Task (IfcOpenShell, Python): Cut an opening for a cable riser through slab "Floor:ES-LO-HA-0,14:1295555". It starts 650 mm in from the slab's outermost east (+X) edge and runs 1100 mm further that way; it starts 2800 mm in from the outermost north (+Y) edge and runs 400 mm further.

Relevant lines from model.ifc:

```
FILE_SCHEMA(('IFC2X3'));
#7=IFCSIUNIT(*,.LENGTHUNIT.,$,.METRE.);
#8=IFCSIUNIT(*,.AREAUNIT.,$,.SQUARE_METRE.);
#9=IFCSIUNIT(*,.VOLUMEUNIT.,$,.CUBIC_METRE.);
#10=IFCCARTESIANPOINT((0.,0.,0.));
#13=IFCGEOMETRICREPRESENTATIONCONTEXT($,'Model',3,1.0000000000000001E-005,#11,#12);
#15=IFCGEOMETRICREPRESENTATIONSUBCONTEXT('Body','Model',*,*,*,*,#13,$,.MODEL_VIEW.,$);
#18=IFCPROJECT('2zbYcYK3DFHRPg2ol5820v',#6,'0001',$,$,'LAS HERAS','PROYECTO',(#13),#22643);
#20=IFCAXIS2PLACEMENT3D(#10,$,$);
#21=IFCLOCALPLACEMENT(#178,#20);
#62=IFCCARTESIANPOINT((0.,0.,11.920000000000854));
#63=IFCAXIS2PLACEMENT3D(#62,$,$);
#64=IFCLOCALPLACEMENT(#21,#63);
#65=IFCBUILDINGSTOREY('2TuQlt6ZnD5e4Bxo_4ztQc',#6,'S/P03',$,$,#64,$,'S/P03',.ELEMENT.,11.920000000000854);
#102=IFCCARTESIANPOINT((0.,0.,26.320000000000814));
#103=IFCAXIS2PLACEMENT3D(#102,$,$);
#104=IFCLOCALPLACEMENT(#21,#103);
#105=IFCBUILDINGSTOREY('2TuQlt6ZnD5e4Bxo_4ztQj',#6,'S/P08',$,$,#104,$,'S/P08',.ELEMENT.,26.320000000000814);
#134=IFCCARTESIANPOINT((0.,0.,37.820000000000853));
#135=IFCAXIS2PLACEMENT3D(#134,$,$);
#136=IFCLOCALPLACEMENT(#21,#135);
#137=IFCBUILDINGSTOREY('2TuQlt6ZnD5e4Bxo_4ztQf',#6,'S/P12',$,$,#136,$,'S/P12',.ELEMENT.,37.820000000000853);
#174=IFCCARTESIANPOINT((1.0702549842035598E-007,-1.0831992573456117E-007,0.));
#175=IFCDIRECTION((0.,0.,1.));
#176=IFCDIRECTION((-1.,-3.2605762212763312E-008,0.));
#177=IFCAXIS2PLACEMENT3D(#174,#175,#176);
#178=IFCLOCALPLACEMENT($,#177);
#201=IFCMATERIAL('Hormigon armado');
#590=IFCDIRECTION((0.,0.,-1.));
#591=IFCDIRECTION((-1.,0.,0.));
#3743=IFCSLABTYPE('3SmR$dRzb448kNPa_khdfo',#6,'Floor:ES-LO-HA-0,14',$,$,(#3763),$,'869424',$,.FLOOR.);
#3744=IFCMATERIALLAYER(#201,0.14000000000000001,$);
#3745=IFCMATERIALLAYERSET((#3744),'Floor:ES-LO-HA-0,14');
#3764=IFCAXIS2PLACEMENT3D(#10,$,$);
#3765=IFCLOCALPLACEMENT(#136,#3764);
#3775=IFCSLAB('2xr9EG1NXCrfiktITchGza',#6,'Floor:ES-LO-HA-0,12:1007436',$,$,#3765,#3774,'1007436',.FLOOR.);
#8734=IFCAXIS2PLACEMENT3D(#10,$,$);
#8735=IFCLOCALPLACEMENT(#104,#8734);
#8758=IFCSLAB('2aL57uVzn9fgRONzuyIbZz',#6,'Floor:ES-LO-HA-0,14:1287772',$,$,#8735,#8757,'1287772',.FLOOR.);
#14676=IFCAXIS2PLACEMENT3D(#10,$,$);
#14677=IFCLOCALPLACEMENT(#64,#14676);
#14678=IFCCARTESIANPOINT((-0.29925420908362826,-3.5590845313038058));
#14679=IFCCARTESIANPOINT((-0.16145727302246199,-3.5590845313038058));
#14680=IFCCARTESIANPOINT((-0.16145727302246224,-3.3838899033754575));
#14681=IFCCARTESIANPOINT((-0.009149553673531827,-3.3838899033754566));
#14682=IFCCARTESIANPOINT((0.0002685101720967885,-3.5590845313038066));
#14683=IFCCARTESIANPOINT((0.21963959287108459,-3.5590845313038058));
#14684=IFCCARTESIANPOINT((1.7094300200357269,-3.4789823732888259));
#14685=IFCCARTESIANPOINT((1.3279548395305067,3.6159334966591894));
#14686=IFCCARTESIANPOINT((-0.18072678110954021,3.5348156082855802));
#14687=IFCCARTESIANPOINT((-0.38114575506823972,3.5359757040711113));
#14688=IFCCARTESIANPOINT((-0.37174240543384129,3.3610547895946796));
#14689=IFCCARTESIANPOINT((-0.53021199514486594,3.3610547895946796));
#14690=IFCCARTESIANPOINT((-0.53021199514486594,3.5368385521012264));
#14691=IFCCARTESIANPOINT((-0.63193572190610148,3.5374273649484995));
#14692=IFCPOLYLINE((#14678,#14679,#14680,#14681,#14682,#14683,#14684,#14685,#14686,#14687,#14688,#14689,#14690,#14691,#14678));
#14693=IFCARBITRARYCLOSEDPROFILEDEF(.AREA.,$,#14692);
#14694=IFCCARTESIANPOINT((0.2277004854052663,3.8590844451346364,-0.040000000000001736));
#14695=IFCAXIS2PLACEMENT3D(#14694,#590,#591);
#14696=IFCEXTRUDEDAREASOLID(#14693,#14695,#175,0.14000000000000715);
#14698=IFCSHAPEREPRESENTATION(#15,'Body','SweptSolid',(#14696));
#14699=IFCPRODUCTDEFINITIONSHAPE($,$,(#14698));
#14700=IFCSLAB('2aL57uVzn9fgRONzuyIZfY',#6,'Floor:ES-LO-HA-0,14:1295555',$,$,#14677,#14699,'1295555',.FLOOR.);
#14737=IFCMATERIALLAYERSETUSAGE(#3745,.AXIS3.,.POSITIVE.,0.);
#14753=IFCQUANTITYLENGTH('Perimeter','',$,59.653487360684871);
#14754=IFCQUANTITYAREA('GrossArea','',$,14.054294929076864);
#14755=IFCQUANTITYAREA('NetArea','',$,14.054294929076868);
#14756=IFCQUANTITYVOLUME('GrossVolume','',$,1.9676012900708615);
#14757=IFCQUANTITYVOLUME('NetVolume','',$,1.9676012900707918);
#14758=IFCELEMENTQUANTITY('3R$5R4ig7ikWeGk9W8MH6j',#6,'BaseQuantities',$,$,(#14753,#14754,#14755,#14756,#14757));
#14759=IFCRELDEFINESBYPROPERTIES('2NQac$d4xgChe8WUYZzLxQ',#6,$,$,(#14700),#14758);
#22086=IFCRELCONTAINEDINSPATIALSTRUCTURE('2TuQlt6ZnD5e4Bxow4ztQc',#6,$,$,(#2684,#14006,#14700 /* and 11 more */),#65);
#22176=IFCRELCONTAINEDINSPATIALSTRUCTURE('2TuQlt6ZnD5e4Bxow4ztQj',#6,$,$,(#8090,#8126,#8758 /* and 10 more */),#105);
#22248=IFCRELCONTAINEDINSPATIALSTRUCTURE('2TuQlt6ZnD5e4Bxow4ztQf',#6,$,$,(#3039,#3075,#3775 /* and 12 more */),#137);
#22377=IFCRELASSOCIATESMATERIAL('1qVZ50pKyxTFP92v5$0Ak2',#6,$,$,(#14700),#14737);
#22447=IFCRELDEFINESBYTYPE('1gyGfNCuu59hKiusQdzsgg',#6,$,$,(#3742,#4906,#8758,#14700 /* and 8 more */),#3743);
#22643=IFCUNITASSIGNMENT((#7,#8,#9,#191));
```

```python
import numpy as np
import ifcopenshell
import ifcopenshell.api.feature
import ifcopenshell.api.geometry
import ifcopenshell.api.pset
import ifcopenshell.api.root
import ifcopenshell.geom
import ifcopenshell.util.element
import ifcopenshell.util.placement
import ifcopenshell.util.representation
import ifcopenshell.util.shape
import ifcopenshell.util.unit

model = ifcopenshell.open("model.ifc")
unit_scale = ifcopenshell.util.unit.calculate_unit_scale(model)
area_scale = ifcopenshell.util.unit.calculate_unit_scale(model, "AREAUNIT")
volume_scale = ifcopenshell.util.unit.calculate_unit_scale(model, "VOLUMEUNIT")
settings = ifcopenshell.geom.settings()


def volume(element):
    """Net volume in cubic metres, openings subtracted."""
    shape = ifcopenshell.geom.create_shape(settings, element)
    return ifcopenshell.util.shape.get_volume(shape.geometry)


slab = model.by_id(14700)
before = volume(slab)

# Extent in the slab's own axes, in metres. The edges named are its -X and -Y sides.
slab_shape = ifcopenshell.geom.create_shape(settings, slab)
vertices = ifcopenshell.util.shape.get_vertices(slab_shape.geometry)
x_min, y_min, bottom = vertices.min(axis=0)
top = vertices[:, 2].max()

opening = ifcopenshell.api.root.create_entity(model, ifc_class="IfcOpeningElement", name="Cable riser opening")
context = ifcopenshell.util.representation.get_context(model, "Model", "Body", "MODEL_VIEW")
width, depth = 1.1, 0.4
outline = [(0.0, 0.0), (width, 0.0), (width, depth), (0.0, depth), (0.0, 0.0)]
# Overshoot both faces by 50 mm so the cut is clean.
shape = ifcopenshell.api.geometry.add_slab_representation(
    model, context=context, depth=top - bottom + 0.1, polyline=outline
)
ifcopenshell.api.geometry.assign_representation(model, product=opening, representation=shape)

matrix = ifcopenshell.util.placement.get_local_placement(slab.ObjectPlacement)
matrix[:, 3] = matrix @ np.append(np.array([x_min + 0.65, y_min + 2.8, bottom - 0.05]) / unit_scale, 1.0)
ifcopenshell.api.geometry.edit_object_placement(model, product=opening, matrix=matrix, is_si=False)
ifcopenshell.api.feature.add_feature(model, feature=opening, element=slab)

after = volume(slab)

# Update the slab's stored quantities.
qto = model.by_id(ifcopenshell.util.element.get_pset(slab, "BaseQuantities", should_inherit=False)["id"])
ifcopenshell.api.pset.edit_qto(model, qto=qto, properties={
    "NetArea": after / (top - bottom) / area_scale,
    "NetVolume": after / volume_scale,
})

print(f"slab volume {before:.3f} -> {after:.3f} m3")

model.write("model_edited.ifc")
```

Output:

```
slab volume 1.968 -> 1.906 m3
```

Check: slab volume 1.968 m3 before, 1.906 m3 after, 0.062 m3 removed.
